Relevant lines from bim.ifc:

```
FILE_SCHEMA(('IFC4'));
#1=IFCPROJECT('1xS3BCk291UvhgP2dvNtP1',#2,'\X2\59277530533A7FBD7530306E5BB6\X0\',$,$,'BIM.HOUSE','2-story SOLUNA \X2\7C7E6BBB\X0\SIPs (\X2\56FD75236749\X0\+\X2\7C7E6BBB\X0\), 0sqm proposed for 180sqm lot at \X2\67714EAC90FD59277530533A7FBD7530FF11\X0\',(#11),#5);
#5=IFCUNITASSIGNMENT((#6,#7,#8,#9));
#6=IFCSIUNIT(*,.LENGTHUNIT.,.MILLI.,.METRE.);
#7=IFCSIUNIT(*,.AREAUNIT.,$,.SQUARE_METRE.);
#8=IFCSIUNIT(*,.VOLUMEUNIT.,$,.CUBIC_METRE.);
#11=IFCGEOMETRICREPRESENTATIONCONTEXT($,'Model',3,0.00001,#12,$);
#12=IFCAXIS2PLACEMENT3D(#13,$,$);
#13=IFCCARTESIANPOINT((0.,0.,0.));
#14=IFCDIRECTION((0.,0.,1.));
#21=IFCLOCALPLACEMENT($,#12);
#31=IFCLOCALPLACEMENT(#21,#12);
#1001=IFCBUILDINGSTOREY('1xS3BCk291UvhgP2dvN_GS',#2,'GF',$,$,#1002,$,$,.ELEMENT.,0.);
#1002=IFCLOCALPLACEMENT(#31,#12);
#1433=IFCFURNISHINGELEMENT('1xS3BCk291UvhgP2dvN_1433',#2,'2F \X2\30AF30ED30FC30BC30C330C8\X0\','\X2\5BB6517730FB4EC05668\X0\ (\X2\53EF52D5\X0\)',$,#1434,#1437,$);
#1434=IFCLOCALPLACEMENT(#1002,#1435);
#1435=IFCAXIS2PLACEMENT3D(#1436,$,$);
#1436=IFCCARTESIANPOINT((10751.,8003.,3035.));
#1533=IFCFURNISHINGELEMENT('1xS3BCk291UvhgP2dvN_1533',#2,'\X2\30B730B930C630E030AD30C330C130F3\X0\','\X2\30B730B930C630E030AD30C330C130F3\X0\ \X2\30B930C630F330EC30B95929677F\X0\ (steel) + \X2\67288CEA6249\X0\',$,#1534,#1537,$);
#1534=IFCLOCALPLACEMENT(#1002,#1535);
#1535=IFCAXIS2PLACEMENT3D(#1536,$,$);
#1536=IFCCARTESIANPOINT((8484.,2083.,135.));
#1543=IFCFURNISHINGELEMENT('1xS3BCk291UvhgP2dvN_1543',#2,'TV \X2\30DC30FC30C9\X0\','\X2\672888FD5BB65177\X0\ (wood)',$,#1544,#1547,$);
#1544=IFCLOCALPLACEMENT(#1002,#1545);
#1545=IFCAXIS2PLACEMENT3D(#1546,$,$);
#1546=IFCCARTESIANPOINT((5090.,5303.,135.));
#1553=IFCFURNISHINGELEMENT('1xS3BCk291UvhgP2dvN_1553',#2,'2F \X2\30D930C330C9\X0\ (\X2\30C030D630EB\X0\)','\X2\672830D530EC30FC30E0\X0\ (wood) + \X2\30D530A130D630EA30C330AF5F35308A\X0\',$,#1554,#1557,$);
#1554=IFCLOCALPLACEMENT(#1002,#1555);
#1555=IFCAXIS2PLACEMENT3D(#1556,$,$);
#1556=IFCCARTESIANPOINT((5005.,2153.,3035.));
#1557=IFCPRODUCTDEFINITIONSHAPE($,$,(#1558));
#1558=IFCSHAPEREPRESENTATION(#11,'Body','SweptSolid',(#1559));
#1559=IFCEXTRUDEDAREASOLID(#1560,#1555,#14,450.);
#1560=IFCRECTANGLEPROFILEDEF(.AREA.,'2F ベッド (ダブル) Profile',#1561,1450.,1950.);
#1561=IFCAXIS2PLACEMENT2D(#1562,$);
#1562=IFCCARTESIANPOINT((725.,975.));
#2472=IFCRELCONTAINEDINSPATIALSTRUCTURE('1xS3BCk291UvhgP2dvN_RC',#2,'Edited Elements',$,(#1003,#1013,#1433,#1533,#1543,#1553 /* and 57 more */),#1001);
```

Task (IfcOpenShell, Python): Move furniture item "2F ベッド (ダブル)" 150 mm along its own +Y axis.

```python
import ifcopenshell
import ifcopenshell.api.geometry
import ifcopenshell.util.placement
import ifcopenshell.util.unit

model = ifcopenshell.open("bim.ifc")
unit_scale = ifcopenshell.util.unit.calculate_unit_scale(model)

item = model.by_guid("1xS3BCk291UvhgP2dvN_1553")
matrix = ifcopenshell.util.placement.get_local_placement(item.ObjectPlacement)
matrix[:3, 3] += matrix[:3, 1] * 0.15 / unit_scale
ifcopenshell.api.geometry.edit_object_placement(model, product=item, matrix=matrix, is_si=False)

print(ifcopenshell.util.placement.get_local_placement(item.ObjectPlacement).round(3) + 0.0)

model.write("bim_edited.ifc")
```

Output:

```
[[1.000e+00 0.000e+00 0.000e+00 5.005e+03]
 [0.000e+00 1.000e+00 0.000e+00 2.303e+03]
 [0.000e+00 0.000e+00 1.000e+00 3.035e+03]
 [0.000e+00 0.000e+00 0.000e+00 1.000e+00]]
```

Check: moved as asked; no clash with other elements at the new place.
